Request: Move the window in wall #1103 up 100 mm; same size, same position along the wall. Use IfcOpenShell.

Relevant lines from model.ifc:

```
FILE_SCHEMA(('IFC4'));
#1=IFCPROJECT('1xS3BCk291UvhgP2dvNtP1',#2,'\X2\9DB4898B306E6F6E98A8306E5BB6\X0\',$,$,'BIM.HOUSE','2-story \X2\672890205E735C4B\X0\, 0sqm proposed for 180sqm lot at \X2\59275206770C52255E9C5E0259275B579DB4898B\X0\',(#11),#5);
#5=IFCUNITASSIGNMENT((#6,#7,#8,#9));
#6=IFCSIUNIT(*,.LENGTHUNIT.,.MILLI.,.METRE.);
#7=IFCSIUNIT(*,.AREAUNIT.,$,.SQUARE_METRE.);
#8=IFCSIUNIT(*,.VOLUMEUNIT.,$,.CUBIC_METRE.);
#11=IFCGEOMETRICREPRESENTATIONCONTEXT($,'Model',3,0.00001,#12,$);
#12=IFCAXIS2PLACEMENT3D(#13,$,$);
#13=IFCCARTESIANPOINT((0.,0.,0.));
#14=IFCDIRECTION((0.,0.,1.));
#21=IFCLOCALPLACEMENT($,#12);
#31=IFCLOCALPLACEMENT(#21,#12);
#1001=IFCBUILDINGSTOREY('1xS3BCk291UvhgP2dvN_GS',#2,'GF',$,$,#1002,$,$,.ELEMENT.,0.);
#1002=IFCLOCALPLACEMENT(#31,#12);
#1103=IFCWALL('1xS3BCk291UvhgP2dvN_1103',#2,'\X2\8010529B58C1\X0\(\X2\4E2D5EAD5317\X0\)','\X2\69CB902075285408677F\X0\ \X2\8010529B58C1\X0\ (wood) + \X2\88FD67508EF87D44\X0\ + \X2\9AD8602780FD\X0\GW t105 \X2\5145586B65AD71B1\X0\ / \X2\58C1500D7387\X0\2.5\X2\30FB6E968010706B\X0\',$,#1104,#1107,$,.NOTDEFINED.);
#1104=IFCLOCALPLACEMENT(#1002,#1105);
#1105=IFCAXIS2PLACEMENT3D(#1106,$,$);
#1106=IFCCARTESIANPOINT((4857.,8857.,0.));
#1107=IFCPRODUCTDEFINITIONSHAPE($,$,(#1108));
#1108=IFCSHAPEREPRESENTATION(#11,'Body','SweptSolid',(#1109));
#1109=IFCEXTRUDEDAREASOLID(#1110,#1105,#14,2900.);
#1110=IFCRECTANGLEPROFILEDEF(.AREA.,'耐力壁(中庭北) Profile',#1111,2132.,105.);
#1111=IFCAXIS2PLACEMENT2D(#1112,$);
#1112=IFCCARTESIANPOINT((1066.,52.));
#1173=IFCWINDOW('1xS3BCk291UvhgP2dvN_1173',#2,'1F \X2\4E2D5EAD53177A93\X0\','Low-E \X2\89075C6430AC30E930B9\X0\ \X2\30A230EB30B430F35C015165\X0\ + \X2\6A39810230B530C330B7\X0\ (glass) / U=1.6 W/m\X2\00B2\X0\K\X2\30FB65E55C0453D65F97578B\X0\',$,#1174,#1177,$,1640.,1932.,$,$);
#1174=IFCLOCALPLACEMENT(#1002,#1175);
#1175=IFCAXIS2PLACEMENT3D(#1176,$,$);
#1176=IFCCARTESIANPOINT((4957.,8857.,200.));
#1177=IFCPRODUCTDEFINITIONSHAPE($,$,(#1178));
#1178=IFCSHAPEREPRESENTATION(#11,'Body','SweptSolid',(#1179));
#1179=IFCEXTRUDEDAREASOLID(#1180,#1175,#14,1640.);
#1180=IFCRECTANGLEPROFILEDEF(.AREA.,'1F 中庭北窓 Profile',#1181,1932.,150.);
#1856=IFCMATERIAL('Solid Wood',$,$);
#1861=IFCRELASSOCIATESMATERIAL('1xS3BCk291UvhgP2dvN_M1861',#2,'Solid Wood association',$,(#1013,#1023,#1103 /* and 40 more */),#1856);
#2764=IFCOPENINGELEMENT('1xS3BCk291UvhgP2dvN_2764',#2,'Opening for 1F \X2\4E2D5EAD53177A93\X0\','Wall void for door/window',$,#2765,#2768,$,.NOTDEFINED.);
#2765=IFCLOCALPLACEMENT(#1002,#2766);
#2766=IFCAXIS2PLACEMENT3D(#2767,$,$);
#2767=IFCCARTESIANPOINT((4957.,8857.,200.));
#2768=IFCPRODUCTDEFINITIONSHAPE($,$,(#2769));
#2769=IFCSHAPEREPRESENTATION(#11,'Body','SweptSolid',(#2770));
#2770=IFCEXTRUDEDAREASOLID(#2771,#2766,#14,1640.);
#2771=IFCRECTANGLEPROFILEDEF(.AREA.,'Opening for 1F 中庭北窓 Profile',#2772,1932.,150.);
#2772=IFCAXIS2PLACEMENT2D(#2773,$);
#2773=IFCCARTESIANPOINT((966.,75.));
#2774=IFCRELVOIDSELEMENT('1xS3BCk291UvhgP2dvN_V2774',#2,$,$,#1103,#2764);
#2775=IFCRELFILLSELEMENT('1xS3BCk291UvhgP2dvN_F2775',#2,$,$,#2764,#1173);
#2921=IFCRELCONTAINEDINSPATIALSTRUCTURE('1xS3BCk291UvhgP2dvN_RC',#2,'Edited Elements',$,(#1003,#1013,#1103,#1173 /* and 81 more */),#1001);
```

```python
import numpy as np
import ifcopenshell
import ifcopenshell.api.geometry
import ifcopenshell.util.placement
import ifcopenshell.util.unit

model = ifcopenshell.open("model.ifc")
unit_scale = ifcopenshell.util.unit.calculate_unit_scale(model)

window = model.by_guid("1xS3BCk291UvhgP2dvN_1173")
opening = window.FillsVoids[0].RelatingOpeningElement
dz = 100.0

shift = np.array([0.0, 0.0, dz])
# The window is not placed relative to its opening, so move both.
for product in (opening, window):
    matrix = ifcopenshell.util.placement.get_local_placement(product.ObjectPlacement)
    matrix[:3, 3] += shift
    ifcopenshell.api.geometry.edit_object_placement(model, product=product, matrix=matrix, is_si=False)

print(f"moved by {dz * unit_scale:+.3f} m")

model.write("model_v2.ifc")
```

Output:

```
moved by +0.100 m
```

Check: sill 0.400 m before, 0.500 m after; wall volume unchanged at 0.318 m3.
